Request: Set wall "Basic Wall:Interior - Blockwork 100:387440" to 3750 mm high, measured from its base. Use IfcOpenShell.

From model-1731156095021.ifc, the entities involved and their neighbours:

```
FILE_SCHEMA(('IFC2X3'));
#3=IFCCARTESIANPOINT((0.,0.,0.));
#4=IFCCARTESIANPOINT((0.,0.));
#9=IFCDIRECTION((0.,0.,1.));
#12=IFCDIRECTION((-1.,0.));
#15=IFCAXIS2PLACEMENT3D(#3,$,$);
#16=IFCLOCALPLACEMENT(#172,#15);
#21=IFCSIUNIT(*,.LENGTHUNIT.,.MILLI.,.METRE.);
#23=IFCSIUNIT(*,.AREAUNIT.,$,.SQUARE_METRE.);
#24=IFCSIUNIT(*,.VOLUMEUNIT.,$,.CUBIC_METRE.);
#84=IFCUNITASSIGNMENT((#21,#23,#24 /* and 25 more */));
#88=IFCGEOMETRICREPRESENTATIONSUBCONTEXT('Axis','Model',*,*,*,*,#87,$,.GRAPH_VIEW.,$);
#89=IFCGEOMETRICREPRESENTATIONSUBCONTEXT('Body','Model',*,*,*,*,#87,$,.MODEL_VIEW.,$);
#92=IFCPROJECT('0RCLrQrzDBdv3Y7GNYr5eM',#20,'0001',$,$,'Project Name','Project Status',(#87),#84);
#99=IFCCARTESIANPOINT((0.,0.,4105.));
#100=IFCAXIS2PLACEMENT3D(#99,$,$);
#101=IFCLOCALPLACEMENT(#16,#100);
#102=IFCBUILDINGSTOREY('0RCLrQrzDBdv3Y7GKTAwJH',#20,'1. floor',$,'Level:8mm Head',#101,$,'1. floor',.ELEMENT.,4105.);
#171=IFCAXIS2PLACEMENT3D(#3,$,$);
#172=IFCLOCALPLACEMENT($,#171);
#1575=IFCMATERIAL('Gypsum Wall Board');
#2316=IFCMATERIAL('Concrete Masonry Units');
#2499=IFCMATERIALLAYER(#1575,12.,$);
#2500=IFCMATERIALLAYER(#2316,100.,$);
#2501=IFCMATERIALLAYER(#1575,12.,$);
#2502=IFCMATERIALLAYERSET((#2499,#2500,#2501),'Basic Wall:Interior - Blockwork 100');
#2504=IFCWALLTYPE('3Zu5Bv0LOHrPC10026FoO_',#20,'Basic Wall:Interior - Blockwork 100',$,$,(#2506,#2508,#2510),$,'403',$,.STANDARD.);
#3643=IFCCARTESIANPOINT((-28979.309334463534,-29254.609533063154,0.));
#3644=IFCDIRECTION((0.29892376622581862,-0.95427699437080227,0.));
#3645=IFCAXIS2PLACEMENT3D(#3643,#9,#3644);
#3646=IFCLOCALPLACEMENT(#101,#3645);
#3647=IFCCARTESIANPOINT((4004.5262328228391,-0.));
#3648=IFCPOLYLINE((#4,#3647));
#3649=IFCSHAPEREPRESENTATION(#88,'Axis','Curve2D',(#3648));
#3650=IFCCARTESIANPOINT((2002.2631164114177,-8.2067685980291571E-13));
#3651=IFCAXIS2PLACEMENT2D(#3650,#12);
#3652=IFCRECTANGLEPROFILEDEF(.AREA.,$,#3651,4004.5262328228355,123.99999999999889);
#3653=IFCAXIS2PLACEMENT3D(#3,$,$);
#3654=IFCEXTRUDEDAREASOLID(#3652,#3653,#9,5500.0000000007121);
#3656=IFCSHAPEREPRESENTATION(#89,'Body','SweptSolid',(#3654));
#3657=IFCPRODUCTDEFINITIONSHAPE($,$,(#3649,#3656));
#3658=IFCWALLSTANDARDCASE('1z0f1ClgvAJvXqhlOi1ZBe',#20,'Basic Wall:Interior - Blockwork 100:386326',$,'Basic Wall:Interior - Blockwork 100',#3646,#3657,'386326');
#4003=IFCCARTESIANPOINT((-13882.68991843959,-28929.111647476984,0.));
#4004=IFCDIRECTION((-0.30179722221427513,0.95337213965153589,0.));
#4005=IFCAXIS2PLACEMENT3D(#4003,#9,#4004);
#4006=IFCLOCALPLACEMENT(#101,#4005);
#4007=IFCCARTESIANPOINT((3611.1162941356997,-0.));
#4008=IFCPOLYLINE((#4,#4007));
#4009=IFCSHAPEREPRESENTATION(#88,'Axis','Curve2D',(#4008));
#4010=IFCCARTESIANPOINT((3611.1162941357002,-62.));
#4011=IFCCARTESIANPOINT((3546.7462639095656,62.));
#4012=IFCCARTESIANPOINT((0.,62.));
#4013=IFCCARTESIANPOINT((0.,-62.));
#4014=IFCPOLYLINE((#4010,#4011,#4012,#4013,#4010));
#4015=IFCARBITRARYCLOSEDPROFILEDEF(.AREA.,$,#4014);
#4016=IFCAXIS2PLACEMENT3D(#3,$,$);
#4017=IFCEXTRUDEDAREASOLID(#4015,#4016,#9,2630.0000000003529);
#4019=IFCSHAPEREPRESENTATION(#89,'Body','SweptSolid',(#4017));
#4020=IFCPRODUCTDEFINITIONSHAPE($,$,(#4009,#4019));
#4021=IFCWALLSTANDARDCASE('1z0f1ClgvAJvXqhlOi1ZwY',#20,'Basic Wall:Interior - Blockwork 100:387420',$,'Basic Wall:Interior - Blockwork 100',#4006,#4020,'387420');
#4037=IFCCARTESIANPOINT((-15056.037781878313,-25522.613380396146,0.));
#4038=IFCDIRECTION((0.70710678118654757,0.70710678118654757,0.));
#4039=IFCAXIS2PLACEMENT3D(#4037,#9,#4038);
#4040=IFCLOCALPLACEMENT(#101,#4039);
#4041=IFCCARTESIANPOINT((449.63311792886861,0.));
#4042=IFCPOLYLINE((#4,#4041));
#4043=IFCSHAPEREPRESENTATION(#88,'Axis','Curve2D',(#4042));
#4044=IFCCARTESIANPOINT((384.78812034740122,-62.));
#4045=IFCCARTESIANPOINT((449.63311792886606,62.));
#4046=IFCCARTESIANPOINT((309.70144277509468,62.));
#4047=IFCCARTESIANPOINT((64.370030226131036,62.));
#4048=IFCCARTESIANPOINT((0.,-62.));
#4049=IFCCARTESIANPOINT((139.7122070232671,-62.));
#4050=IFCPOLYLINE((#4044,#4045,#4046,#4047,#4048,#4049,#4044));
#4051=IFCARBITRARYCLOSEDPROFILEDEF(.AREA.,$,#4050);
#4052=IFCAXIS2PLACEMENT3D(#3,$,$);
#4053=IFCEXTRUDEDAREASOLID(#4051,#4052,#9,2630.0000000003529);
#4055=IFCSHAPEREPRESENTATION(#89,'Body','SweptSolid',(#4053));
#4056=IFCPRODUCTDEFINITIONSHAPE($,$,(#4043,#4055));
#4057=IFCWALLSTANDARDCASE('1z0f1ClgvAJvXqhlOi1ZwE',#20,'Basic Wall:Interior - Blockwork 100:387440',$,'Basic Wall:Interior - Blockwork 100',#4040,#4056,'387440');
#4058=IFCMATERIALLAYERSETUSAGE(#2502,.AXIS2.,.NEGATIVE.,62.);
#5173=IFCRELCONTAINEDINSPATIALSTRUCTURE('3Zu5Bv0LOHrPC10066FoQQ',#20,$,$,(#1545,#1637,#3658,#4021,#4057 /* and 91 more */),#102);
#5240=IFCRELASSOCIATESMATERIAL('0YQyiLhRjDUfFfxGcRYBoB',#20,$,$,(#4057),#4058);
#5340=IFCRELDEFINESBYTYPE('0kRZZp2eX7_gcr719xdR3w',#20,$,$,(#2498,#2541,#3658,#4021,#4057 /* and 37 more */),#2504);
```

```python
import ifcopenshell
import ifcopenshell.geom
import ifcopenshell.util.representation
import ifcopenshell.util.shape
import ifcopenshell.util.unit

model = ifcopenshell.open("model-1731156095021.ifc")
unit_scale = ifcopenshell.util.unit.calculate_unit_scale(model)
settings = ifcopenshell.geom.settings()


def volume(element):
    """Net volume in cubic metres, openings subtracted."""
    shape = ifcopenshell.geom.create_shape(settings, element)
    return ifcopenshell.util.shape.get_volume(shape.geometry)


wall = model.by_guid("1z0f1ClgvAJvXqhlOi1ZwE")
before = volume(wall)

body = ifcopenshell.util.representation.get_representation(wall, "Model", "Body")
solid = body.Items[0]
old_height = solid.Depth
solid.Depth = 3.75 / unit_scale
after = volume(wall)

print(f"height {old_height:g} -> {solid.Depth:g}, volume {before:.3f} -> {after:.3f} m3")

model.write("model-1731156095021_edited.ifc")
```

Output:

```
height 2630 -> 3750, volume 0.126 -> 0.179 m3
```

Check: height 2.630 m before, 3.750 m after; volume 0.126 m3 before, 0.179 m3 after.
